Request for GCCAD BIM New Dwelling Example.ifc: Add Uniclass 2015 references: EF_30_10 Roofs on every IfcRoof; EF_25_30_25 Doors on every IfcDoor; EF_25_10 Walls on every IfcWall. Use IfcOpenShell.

First a look at what the model holds.

```python
import ifcopenshell

model = ifcopenshell.open("GCCAD BIM New Dwelling Example.ifc")
print(model.schema)
print("classifications:", [c.Name for c in model.by_type("IfcClassification")])
for ifc_class in ("IfcDoor", "IfcRoof", "IfcStair", "IfcWall", "IfcWindow"):
    print(ifc_class, len(model.by_type(ifc_class)))
```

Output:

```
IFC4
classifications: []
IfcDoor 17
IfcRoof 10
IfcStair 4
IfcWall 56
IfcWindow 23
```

```python
import ifcopenshell
import ifcopenshell.api.classification

model = ifcopenshell.open("GCCAD BIM New Dwelling Example.ifc")

system = ifcopenshell.api.classification.add_classification(model, classification="Uniclass 2015")

codes = {
    "IfcRoof": ("EF_30_10", "Roofs"),
    "IfcDoor": ("EF_25_30_25", "Doors"),
    "IfcWall": ("EF_25_10", "Walls"),
}
for ifc_class, (code, name) in codes.items():
    products = model.by_type(ifc_class)
    ifcopenshell.api.classification.add_reference(
        model, products=products, classification=system, identification=code, name=name
    )
    print(code, len(products))

model.write("GCCAD BIM New Dwelling Example_updated.ifc")
```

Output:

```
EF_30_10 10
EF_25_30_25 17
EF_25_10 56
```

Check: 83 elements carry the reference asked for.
